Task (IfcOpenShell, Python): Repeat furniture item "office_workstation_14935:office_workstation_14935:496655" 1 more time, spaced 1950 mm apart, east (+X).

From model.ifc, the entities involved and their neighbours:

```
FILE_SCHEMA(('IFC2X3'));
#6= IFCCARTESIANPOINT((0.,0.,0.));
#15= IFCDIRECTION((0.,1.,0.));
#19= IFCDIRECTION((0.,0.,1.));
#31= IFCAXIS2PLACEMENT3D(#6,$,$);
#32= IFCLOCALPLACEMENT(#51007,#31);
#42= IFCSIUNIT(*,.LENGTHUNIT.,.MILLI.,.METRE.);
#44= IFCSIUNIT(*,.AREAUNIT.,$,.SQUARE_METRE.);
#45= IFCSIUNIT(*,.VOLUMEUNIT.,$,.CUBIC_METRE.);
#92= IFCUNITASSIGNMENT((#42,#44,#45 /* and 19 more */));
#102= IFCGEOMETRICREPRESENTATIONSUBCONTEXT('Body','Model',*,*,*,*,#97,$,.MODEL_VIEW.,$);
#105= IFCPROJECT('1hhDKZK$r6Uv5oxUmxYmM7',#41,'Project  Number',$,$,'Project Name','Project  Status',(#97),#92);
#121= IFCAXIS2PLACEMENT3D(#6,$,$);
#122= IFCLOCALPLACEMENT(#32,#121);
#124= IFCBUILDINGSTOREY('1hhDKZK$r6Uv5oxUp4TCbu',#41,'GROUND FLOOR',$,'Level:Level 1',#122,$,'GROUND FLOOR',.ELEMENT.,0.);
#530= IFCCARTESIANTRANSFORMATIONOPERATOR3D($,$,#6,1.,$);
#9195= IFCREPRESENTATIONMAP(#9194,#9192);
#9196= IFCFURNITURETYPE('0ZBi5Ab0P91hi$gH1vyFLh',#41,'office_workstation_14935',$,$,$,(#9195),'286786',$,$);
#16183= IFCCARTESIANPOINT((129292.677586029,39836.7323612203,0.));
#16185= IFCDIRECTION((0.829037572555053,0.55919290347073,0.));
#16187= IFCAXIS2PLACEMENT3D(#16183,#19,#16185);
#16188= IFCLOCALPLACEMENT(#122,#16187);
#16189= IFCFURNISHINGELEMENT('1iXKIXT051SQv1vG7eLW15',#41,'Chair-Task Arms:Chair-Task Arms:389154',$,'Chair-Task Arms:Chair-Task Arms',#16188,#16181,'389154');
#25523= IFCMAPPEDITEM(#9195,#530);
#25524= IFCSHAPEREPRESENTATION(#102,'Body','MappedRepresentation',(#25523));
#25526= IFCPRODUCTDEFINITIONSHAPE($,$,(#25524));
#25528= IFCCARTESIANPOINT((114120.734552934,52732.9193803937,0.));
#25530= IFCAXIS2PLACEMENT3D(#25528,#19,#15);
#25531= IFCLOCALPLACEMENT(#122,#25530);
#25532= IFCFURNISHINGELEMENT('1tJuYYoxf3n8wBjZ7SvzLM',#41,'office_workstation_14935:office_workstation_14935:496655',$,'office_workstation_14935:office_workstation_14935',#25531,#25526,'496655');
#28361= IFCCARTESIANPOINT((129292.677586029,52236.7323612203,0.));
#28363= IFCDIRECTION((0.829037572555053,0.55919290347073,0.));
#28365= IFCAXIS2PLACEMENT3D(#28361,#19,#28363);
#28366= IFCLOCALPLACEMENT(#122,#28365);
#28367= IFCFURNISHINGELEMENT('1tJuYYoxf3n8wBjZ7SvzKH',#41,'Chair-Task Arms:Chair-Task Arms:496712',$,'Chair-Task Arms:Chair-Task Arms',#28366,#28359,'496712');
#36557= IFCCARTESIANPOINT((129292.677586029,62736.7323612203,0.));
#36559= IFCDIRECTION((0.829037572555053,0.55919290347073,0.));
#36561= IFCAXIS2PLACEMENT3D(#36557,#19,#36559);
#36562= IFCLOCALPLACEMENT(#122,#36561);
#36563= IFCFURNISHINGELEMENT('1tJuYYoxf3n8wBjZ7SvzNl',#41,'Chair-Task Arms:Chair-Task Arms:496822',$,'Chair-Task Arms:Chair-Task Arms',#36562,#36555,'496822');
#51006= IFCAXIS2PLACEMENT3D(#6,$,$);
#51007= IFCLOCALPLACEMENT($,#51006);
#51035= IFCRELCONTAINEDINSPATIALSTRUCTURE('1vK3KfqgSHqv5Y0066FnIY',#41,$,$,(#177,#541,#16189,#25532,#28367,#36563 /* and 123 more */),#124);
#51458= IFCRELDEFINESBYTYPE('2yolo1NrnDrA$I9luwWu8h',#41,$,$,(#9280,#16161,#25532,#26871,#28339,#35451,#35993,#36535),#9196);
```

```python
import numpy as np
import ifcopenshell
import ifcopenshell.api.geometry
import ifcopenshell.api.root
import ifcopenshell.util.element
import ifcopenshell.util.placement
import ifcopenshell.util.unit

model = ifcopenshell.open("model.ifc")
unit_scale = ifcopenshell.util.unit.calculate_unit_scale(model)


def reuse_history(source, copy):
    """copy_class also copies each property set's owner history, people and application; keep the originals."""
    for rel in copy.IsDefinedBy:
        if rel.is_a("IfcRelDefinesByProperties") and (history := rel.RelatingPropertyDefinition.OwnerHistory):
            rel.RelatingPropertyDefinition.OwnerHistory = source.OwnerHistory
            ifcopenshell.util.element.remove_deep2(model, history)


source = model.by_guid("1tJuYYoxf3n8wBjZ7SvzLM")
base = ifcopenshell.util.placement.get_local_placement(source.ObjectPlacement)
step = np.array([1.0, 0.0, 0.0]) * 1.95 / unit_scale

for i in range(1, 2):
    copy = ifcopenshell.api.root.copy_class(model, product=source)
    copy.Representation = ifcopenshell.util.element.copy_deep(
        model, source.Representation, exclude=["IfcGeometricRepresentationContext", "IfcRepresentationMap"]
    )
    copy.Name = "office_workstation_14935:office_workstation_14935"
    copy.Tag = None
    reuse_history(source, copy)
    matrix = base.copy()
    matrix[:3, 3] += i * step
    print("added at", matrix[:3, 3].round(3) + 0.0)
    ifcopenshell.api.geometry.edit_object_placement(model, product=copy, matrix=matrix, is_si=False)

model.write("model_edited.ifc")
```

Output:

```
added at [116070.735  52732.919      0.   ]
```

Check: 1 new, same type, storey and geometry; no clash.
